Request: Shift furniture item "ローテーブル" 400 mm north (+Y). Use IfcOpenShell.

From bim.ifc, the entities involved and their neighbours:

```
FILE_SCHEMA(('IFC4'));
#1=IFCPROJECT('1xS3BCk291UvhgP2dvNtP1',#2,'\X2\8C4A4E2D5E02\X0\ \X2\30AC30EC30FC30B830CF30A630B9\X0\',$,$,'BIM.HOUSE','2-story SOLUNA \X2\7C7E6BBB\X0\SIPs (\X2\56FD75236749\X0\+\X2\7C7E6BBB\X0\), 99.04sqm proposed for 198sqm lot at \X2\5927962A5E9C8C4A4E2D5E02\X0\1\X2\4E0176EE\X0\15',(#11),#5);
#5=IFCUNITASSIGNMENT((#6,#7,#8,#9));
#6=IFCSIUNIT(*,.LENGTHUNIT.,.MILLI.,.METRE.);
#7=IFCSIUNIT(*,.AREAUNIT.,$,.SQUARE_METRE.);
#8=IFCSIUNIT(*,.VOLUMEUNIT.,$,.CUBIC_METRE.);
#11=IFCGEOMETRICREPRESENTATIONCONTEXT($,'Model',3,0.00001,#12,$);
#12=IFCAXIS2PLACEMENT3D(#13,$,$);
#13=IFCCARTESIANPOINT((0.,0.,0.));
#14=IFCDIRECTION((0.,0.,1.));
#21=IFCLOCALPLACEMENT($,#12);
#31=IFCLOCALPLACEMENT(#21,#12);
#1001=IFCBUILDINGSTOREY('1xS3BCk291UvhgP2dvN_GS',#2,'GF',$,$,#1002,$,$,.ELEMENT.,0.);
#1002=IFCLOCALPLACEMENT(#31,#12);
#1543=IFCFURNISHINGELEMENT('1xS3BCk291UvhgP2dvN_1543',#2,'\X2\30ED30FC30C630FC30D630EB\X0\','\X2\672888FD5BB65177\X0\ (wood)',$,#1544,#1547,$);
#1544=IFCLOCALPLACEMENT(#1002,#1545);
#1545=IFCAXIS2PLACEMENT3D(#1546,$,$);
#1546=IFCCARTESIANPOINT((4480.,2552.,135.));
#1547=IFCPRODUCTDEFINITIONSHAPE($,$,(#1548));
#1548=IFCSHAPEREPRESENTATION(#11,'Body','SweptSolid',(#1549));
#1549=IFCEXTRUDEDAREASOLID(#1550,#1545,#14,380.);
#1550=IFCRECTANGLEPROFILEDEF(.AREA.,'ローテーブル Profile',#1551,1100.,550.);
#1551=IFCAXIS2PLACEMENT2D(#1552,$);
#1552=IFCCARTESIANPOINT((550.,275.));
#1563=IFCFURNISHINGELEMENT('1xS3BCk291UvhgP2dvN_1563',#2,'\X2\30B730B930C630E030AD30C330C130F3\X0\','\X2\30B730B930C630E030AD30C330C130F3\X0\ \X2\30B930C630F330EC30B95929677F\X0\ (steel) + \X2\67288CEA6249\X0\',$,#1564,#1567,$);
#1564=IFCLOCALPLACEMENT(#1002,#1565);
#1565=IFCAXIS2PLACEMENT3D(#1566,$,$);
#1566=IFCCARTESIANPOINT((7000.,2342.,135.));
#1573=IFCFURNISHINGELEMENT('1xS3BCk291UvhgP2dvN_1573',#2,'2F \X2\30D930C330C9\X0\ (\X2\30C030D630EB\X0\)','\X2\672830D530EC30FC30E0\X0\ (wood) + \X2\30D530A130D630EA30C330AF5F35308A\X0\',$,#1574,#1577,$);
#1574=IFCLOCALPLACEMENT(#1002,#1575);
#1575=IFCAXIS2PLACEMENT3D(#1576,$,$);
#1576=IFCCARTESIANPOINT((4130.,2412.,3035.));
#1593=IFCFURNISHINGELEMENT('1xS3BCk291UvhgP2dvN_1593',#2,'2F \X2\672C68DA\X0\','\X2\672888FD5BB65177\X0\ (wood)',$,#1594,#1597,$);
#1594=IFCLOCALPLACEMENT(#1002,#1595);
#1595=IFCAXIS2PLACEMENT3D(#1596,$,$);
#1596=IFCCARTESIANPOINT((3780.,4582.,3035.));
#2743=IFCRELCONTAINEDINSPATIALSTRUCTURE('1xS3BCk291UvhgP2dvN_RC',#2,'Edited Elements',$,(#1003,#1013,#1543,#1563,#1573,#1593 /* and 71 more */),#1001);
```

```python
import ifcopenshell
import ifcopenshell.api.geometry
import ifcopenshell.util.placement

model = ifcopenshell.open("bim.ifc")

item = model.by_guid("1xS3BCk291UvhgP2dvN_1543")
matrix = ifcopenshell.util.placement.get_local_placement(item.ObjectPlacement)
matrix[1, 3] += 400.0
ifcopenshell.api.geometry.edit_object_placement(model, product=item, matrix=matrix, is_si=False)

print(ifcopenshell.util.placement.get_local_placement(item.ObjectPlacement).round(3) + 0.0)

model.write("bim-out.ifc")
```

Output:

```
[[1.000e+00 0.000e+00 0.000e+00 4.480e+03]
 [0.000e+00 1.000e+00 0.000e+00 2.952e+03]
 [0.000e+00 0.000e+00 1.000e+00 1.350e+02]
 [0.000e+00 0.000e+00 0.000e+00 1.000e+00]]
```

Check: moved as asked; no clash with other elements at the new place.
